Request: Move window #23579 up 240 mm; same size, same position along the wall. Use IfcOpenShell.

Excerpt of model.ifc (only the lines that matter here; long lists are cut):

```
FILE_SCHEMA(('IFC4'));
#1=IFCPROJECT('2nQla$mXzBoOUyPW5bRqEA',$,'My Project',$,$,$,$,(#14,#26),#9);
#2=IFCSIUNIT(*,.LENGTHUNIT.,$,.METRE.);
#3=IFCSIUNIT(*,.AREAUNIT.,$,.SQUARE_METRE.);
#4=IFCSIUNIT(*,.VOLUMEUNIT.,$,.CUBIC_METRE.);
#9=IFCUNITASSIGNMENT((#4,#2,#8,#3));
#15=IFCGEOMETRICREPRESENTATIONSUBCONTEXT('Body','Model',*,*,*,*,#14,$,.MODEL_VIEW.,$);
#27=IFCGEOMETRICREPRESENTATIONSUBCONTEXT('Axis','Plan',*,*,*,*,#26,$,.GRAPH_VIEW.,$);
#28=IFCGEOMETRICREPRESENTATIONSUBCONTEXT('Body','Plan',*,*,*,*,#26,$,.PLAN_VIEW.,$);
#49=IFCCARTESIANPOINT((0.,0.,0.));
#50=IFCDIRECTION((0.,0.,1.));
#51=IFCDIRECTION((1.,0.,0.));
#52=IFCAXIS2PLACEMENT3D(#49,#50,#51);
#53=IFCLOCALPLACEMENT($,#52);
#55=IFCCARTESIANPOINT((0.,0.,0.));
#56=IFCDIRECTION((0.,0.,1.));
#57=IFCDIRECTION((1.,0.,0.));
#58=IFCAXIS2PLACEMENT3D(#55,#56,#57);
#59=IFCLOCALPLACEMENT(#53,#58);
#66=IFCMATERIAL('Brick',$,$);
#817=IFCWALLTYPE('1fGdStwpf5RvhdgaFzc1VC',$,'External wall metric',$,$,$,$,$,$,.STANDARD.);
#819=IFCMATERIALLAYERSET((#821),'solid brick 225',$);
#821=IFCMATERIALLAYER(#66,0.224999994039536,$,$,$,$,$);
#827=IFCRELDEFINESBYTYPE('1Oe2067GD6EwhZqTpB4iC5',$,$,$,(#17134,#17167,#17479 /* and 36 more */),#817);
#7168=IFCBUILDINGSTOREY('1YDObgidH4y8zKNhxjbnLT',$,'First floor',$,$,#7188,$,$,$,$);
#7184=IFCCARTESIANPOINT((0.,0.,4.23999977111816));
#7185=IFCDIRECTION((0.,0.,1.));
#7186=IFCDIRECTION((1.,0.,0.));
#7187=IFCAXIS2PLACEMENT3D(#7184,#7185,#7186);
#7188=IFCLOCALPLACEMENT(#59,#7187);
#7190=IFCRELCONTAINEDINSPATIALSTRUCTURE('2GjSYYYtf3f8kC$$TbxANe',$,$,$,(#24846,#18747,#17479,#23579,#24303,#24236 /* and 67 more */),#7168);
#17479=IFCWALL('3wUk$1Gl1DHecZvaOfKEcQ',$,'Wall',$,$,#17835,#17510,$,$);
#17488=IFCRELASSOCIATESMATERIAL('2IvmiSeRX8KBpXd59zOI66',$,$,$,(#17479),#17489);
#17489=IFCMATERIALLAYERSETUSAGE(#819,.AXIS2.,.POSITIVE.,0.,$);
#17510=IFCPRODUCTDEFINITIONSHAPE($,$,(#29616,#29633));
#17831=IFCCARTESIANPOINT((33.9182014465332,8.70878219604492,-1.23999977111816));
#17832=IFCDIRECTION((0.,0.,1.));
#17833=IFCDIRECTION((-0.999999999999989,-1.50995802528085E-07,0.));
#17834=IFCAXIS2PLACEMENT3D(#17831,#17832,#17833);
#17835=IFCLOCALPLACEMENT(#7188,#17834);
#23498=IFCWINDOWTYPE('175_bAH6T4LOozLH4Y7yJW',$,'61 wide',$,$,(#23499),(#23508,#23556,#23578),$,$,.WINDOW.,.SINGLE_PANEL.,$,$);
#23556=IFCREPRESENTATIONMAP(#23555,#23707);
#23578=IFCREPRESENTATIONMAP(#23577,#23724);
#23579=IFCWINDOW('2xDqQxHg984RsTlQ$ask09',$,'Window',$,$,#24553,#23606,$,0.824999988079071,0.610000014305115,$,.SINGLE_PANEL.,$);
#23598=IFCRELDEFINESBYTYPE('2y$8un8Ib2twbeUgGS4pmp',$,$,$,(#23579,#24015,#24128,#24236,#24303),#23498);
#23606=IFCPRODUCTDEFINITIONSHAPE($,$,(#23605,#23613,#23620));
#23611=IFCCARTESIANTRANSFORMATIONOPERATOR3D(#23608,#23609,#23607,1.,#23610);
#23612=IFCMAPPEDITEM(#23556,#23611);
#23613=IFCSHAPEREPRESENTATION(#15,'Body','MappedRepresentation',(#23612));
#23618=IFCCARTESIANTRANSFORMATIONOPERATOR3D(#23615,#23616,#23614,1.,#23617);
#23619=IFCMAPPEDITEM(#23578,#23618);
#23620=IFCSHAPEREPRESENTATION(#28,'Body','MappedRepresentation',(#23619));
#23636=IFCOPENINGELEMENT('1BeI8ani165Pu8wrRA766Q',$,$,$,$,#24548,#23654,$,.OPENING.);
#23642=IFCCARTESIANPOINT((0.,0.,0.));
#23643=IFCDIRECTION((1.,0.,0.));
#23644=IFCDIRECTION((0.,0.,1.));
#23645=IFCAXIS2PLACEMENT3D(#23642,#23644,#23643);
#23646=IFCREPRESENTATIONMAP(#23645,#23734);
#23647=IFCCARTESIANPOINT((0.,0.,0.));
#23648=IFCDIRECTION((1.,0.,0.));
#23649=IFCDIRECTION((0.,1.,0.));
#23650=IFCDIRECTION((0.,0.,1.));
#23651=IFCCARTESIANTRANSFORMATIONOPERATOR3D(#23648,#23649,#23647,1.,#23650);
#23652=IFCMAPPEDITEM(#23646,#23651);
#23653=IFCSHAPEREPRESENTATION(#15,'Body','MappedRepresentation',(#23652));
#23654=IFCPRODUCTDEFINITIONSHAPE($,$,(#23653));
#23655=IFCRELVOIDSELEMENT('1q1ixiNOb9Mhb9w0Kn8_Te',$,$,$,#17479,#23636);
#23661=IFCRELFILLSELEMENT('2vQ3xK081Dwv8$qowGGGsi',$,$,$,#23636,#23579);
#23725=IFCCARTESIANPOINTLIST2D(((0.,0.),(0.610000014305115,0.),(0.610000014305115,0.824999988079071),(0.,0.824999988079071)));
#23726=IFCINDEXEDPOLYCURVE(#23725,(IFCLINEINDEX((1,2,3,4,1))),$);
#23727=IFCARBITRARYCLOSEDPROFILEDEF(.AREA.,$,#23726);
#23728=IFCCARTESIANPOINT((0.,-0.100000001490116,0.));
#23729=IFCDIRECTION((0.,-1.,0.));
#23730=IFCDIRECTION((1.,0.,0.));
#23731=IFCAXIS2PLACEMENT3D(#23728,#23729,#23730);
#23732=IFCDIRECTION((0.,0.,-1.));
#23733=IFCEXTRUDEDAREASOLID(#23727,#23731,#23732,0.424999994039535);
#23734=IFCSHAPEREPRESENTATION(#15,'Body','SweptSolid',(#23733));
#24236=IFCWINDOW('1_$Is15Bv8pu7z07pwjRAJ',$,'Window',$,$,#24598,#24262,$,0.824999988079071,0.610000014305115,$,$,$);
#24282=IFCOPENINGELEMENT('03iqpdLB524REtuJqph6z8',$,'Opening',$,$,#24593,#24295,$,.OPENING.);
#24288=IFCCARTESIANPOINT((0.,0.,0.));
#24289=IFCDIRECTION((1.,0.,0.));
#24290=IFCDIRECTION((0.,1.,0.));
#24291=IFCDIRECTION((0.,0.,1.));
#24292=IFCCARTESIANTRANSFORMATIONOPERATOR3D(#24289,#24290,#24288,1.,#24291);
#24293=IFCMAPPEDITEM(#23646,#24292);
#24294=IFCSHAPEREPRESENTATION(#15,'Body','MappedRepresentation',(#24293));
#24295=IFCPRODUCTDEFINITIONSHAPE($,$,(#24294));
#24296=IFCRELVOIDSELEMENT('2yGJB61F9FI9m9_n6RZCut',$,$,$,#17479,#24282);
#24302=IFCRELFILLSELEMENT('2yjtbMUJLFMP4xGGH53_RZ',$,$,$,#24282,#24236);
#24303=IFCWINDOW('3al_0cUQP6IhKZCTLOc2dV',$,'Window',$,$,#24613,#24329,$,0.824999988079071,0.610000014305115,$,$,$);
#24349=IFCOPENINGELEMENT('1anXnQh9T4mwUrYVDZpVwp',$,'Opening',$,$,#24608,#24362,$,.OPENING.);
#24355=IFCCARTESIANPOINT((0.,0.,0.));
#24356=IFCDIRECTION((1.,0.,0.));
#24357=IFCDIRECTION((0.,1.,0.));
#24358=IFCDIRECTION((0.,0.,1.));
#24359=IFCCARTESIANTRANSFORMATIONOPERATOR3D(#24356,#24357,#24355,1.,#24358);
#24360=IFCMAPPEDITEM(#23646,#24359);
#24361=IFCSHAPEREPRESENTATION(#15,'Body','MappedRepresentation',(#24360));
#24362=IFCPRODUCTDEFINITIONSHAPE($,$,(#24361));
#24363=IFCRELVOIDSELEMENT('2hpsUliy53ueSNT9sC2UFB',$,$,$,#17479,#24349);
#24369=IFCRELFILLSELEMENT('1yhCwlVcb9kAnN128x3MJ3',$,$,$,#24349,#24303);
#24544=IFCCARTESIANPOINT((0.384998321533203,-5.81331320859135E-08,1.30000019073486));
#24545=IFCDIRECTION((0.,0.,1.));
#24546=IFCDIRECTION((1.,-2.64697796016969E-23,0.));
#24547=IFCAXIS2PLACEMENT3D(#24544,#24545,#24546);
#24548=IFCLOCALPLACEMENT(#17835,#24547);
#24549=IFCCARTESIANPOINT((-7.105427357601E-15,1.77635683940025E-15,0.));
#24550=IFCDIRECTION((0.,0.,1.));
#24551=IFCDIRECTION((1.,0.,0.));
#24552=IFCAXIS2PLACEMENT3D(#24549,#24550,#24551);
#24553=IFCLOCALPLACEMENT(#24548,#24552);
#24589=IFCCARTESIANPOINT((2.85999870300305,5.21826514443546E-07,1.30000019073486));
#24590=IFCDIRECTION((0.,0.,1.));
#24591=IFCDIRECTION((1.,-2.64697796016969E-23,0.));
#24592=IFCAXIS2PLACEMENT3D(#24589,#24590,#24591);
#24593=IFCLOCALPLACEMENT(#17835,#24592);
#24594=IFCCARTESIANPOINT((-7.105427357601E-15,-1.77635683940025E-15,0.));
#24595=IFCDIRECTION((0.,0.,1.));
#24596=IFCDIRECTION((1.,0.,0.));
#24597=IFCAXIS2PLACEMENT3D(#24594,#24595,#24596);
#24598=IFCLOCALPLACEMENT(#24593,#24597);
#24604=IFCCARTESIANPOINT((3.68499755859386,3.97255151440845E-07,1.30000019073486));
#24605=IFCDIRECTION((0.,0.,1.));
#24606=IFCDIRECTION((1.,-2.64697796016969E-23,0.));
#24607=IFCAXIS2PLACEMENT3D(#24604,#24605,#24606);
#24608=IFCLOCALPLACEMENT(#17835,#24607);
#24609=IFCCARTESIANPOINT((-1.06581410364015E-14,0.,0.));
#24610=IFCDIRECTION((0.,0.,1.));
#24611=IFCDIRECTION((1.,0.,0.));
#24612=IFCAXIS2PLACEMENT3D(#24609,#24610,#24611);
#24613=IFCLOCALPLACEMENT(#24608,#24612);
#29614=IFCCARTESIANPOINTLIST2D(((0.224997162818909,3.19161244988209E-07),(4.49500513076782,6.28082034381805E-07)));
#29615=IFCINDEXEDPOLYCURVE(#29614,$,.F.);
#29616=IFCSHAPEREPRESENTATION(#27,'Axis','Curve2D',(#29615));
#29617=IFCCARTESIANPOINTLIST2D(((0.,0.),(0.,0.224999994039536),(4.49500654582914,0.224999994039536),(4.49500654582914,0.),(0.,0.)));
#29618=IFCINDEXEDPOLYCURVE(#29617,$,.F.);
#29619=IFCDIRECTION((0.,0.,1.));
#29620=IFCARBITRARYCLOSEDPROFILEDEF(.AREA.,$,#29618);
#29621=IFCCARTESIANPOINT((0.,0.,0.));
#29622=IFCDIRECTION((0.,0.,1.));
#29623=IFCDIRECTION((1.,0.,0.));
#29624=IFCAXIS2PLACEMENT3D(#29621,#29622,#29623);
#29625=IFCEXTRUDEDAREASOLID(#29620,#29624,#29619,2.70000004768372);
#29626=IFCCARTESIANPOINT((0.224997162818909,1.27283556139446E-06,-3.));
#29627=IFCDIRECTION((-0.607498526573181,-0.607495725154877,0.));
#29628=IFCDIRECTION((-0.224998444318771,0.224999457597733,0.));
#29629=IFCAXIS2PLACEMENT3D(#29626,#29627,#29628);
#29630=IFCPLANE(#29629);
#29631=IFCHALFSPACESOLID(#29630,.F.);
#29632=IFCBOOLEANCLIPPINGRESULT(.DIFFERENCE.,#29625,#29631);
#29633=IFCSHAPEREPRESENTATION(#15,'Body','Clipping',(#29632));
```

```python
import numpy as np
import ifcopenshell
import ifcopenshell.api.geometry
import ifcopenshell.util.placement
import ifcopenshell.util.unit

model = ifcopenshell.open("model.ifc")
unit_scale = ifcopenshell.util.unit.calculate_unit_scale(model)

window = model.by_guid("2xDqQxHg984RsTlQ$ask09")
opening = window.FillsVoids[0].RelatingOpeningElement
dz = 0.24

shift = np.array([0.0, 0.0, dz])
# The window is placed relative to its opening, so it follows when the opening moves.
matrix = ifcopenshell.util.placement.get_local_placement(opening.ObjectPlacement)
matrix[:3, 3] += shift
ifcopenshell.api.geometry.edit_object_placement(
    model, product=opening, matrix=matrix, is_si=False, should_transform_children=True
)

print(f"moved by {dz * unit_scale:+.3f} m")

model.write("model_v2.ifc")
```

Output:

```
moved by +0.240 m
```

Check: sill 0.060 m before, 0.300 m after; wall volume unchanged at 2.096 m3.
